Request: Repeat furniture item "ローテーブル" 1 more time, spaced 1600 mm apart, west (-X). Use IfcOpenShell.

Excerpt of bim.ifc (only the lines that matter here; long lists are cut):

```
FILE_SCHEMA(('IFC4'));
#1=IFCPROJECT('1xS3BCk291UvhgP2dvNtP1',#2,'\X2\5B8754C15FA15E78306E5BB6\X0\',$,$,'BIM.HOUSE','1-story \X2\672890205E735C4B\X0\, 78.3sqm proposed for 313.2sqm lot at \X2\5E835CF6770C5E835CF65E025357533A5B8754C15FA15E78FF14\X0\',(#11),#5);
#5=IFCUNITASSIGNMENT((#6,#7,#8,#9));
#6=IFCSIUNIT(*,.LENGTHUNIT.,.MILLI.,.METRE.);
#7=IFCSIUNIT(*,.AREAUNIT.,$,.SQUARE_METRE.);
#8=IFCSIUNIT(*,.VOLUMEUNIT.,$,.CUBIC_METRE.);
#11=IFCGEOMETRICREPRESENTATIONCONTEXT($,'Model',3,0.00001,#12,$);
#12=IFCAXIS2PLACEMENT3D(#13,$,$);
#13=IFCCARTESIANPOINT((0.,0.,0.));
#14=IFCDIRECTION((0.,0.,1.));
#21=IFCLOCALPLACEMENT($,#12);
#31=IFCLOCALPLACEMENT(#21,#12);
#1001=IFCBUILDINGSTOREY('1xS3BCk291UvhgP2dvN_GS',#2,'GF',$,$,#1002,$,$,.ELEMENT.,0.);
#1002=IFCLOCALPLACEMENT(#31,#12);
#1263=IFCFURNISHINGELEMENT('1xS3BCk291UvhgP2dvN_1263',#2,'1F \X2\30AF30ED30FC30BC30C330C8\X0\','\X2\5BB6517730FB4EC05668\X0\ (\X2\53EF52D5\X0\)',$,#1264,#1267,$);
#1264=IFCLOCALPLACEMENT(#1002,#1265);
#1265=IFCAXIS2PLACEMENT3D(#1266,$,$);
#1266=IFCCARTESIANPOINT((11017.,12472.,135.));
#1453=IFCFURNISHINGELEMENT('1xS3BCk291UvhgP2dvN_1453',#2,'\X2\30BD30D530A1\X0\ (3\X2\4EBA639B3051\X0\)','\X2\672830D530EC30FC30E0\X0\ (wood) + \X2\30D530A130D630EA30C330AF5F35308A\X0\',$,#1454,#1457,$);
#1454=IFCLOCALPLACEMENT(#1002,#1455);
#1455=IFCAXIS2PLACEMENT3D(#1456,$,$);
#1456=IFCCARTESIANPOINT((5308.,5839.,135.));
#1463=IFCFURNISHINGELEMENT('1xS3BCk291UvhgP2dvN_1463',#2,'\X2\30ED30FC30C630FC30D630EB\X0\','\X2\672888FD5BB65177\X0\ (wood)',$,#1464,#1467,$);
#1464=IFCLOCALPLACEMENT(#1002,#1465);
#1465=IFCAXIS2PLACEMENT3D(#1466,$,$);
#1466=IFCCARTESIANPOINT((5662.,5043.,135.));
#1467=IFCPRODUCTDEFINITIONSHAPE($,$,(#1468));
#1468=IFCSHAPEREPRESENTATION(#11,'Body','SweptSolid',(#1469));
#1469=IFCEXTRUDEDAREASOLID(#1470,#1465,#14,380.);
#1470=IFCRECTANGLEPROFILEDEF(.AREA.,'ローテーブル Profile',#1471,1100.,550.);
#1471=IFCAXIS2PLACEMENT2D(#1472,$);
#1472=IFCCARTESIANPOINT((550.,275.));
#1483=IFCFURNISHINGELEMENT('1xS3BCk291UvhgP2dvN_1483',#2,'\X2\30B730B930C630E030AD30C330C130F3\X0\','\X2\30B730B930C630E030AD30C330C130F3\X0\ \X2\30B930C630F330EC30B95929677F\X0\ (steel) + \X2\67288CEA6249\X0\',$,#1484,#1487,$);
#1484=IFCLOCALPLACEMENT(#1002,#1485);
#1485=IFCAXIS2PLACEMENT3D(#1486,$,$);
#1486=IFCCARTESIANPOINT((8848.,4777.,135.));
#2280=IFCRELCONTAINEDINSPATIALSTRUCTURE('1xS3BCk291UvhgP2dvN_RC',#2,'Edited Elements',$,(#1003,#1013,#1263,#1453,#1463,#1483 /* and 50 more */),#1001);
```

```python
import numpy as np
import ifcopenshell
import ifcopenshell.api.geometry
import ifcopenshell.api.root
import ifcopenshell.util.element
import ifcopenshell.util.placement

model = ifcopenshell.open("bim.ifc")


def reuse_history(source, copy):
    """copy_class also copies each property set's owner history, people and application; keep the originals."""
    for rel in copy.IsDefinedBy:
        if rel.is_a("IfcRelDefinesByProperties") and (history := rel.RelatingPropertyDefinition.OwnerHistory):
            rel.RelatingPropertyDefinition.OwnerHistory = source.OwnerHistory
            ifcopenshell.util.element.remove_deep2(model, history)


source = model.by_guid("1xS3BCk291UvhgP2dvN_1463")
base = ifcopenshell.util.placement.get_local_placement(source.ObjectPlacement)
step = np.array([-1.0, 0.0, 0.0]) * 1600.0

for i in range(1, 2):
    copy = ifcopenshell.api.root.copy_class(model, product=source)
    copy.Representation = ifcopenshell.util.element.copy_deep(
        model, source.Representation, exclude=["IfcGeometricRepresentationContext", "IfcRepresentationMap"]
    )
    reuse_history(source, copy)
    matrix = base.copy()
    matrix[:3, 3] += i * step
    print("added at", matrix[:3, 3].round(3) + 0.0)
    ifcopenshell.api.geometry.edit_object_placement(model, product=copy, matrix=matrix, is_si=False)

model.write("bim_rev.ifc")
```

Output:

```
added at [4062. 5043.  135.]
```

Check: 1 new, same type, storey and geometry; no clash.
